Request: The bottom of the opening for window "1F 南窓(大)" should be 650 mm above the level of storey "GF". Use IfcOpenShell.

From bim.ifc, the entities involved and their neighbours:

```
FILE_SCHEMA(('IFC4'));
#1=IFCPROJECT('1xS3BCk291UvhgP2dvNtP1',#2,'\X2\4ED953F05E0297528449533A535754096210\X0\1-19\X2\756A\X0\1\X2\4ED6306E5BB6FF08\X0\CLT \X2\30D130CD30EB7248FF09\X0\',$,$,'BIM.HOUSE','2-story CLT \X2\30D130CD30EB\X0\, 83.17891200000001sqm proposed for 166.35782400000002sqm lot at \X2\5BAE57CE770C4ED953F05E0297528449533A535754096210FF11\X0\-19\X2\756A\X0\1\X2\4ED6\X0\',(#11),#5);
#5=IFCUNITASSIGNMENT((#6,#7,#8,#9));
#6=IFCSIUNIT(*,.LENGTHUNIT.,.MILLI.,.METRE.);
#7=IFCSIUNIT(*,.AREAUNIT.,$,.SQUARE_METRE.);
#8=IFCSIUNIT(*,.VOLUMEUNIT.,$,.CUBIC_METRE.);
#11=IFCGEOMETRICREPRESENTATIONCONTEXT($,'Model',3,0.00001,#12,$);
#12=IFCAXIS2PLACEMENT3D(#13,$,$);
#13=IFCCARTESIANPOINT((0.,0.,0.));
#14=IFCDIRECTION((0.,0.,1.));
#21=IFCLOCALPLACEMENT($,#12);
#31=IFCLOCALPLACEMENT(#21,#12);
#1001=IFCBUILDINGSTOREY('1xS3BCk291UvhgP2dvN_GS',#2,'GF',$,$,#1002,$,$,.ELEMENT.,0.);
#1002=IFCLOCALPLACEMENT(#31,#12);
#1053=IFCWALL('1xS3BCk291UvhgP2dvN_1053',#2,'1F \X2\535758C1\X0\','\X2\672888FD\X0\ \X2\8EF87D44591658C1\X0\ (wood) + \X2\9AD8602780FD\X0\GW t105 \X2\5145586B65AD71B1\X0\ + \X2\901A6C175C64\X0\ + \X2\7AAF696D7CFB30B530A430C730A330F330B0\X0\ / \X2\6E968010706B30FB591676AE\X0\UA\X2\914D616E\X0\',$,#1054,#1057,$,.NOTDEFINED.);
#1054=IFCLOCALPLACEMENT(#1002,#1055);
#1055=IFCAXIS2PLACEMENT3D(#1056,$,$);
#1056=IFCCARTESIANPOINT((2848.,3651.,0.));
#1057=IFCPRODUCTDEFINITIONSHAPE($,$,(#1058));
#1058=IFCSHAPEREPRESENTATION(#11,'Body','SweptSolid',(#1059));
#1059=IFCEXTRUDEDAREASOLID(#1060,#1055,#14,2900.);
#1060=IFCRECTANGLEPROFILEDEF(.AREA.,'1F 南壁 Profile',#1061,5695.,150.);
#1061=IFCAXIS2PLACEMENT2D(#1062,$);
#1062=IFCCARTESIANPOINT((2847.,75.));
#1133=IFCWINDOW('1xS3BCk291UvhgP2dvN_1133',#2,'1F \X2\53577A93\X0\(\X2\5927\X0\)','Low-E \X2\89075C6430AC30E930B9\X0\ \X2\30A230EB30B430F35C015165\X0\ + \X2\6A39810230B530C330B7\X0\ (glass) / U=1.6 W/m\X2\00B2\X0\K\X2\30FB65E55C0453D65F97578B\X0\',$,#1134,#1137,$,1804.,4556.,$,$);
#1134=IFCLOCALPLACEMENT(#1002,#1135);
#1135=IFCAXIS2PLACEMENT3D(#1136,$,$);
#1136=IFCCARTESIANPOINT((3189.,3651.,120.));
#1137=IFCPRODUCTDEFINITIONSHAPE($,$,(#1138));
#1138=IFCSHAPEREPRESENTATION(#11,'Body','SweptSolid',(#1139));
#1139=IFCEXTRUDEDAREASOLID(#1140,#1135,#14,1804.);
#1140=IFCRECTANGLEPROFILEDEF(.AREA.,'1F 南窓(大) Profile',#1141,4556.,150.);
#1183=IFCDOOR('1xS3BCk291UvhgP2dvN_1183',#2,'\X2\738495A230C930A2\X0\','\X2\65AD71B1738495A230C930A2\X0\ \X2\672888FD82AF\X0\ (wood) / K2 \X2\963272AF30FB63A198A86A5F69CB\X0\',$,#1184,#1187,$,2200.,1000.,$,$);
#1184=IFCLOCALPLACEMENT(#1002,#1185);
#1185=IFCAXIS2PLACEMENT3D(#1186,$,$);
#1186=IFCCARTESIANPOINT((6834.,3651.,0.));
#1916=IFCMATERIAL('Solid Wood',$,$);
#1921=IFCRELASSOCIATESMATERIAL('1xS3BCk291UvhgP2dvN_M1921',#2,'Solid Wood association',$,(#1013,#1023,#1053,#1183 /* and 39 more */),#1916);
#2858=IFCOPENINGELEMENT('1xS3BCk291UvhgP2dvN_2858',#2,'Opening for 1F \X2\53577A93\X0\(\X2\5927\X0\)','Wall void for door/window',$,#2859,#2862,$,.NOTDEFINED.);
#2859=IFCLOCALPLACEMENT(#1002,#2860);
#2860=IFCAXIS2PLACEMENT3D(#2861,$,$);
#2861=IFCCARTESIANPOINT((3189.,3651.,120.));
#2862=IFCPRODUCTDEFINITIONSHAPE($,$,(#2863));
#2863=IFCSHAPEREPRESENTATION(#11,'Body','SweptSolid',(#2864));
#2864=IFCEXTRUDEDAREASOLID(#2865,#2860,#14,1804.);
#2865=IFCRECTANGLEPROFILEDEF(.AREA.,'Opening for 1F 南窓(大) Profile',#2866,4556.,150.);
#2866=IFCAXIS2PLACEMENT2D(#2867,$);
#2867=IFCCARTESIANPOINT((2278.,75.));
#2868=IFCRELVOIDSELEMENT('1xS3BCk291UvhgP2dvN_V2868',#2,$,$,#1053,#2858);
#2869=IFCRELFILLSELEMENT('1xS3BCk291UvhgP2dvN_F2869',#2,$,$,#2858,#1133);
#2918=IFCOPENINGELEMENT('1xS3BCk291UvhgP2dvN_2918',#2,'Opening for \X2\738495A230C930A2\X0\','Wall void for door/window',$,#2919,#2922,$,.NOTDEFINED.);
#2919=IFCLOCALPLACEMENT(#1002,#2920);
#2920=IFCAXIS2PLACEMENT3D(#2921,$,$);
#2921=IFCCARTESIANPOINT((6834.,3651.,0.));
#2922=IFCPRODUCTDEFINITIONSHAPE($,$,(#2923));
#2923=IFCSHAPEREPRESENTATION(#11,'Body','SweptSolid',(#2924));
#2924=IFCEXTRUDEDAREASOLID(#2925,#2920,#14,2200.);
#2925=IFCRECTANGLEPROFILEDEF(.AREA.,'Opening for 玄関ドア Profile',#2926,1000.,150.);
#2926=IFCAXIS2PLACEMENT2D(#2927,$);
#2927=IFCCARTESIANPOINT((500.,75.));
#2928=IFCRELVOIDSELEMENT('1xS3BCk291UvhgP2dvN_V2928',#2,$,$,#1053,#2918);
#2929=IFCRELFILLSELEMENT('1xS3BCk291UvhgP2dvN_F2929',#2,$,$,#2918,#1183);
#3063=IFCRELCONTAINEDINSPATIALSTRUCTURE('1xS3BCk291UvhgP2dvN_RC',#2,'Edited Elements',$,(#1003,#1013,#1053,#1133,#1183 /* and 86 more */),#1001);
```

```python
import numpy as np
import ifcopenshell
import ifcopenshell.api.geometry
import ifcopenshell.geom
import ifcopenshell.util.element
import ifcopenshell.util.placement
import ifcopenshell.util.shape
import ifcopenshell.util.unit

model = ifcopenshell.open("bim.ifc")
unit_scale = ifcopenshell.util.unit.calculate_unit_scale(model)

window = model.by_guid("1xS3BCk291UvhgP2dvN_1133")
opening = window.FillsVoids[0].RelatingOpeningElement
storey = ifcopenshell.util.element.get_container(window, ifc_class="IfcBuildingStorey")
level = ifcopenshell.util.placement.get_local_placement(storey.ObjectPlacement)[2, 3]

# The opening's origin need not be at the sill, so measure its lowest point.
shape = ifcopenshell.geom.create_shape(ifcopenshell.geom.settings(), opening)
bottom = ifcopenshell.util.shape.get_shape_bottom_elevation(shape, shape.geometry) / unit_scale
dz = level + 650.0 - bottom

shift = np.array([0.0, 0.0, dz])
# The window is not placed relative to its opening, so move both.
for product in (opening, window):
    matrix = ifcopenshell.util.placement.get_local_placement(product.ObjectPlacement)
    matrix[:3, 3] += shift
    ifcopenshell.api.geometry.edit_object_placement(model, product=product, matrix=matrix, is_si=False)

print(f"moved by {dz * unit_scale:+.3f} m")

model.write("bim_v2.ifc")
```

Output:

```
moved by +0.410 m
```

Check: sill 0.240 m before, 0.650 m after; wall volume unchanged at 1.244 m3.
